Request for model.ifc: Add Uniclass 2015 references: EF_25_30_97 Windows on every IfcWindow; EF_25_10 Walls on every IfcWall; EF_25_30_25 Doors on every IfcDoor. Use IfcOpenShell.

First a look at what the model holds.

```python
import ifcopenshell

model = ifcopenshell.open("model.ifc")
print(model.schema)
print("classifications:", [c.Name for c in model.by_type("IfcClassification")])
for ifc_class in ("IfcDoor", "IfcRoof", "IfcStair", "IfcWall", "IfcWindow"):
    print(ifc_class, len(model.by_type(ifc_class)))
```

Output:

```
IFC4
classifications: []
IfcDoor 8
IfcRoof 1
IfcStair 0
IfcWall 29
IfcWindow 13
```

```python
import ifcopenshell
import ifcopenshell.api.classification

model = ifcopenshell.open("model.ifc")

system = ifcopenshell.api.classification.add_classification(model, classification="Uniclass 2015")

codes = {
    "IfcWindow": ("EF_25_30_97", "Windows"),
    "IfcWall": ("EF_25_10", "Walls"),
    "IfcDoor": ("EF_25_30_25", "Doors"),
}
for ifc_class, (code, name) in codes.items():
    products = model.by_type(ifc_class)
    ifcopenshell.api.classification.add_reference(
        model, products=products, classification=system, identification=code, name=name
    )
    print(code, len(products))

model.write("model-out.ifc")
```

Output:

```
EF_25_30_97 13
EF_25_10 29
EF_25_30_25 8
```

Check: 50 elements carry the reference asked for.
